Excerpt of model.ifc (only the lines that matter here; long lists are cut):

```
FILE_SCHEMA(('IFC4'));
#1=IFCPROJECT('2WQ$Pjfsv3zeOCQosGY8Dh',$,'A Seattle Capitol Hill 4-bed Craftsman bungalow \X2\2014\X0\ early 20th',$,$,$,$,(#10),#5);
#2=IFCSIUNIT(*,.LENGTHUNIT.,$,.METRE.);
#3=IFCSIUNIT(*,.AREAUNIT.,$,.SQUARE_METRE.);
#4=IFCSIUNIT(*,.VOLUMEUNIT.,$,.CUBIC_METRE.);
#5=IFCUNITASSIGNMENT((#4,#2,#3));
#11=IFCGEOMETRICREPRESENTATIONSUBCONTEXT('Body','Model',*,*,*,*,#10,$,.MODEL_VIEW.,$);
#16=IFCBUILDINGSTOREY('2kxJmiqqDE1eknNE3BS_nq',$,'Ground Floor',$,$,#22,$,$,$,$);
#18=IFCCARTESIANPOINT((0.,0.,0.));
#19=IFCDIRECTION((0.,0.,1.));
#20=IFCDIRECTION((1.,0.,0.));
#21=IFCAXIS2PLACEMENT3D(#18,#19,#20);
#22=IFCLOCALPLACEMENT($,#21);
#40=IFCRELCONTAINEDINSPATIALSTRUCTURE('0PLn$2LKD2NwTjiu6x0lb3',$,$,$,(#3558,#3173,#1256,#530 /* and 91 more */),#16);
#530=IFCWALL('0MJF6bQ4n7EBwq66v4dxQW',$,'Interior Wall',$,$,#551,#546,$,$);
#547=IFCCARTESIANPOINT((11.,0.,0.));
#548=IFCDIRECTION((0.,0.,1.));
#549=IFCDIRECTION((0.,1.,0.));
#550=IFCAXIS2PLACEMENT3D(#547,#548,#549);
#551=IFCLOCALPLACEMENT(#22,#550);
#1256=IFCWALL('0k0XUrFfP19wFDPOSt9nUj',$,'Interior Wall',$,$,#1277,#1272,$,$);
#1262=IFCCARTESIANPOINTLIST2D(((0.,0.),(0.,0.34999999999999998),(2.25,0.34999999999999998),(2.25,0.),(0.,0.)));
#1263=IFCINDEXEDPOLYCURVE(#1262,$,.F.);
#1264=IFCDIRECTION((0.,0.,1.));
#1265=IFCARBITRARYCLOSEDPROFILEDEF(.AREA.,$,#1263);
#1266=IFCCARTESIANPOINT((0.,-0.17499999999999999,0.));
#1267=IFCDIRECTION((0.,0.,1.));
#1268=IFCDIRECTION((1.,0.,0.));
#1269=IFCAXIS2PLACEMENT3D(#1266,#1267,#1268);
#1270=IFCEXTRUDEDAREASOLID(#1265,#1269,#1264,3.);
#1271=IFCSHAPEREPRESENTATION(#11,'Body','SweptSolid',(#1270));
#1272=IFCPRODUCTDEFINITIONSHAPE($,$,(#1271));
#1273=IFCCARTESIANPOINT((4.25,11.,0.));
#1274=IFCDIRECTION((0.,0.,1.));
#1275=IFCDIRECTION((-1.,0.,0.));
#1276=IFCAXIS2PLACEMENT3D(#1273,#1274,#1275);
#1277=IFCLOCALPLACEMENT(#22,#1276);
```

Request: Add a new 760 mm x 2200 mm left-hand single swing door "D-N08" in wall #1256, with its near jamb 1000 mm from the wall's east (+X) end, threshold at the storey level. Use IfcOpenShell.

```python
import numpy as np
import ifcopenshell
import ifcopenshell.api.feature
import ifcopenshell.api.geometry
import ifcopenshell.api.root
import ifcopenshell.api.spatial
import ifcopenshell.geom
import ifcopenshell.util.element
import ifcopenshell.util.placement
import ifcopenshell.util.representation
import ifcopenshell.util.shape
import ifcopenshell.util.unit

model = ifcopenshell.open("model.ifc")
unit_scale = ifcopenshell.util.unit.calculate_unit_scale(model)
settings = ifcopenshell.geom.settings()


def volume(element):
    """Net volume in cubic metres, openings subtracted."""
    shape = ifcopenshell.geom.create_shape(settings, element)
    return ifcopenshell.util.shape.get_volume(shape.geometry)


wall = model.by_guid("0k0XUrFfP19wFDPOSt9nUj")
storey = ifcopenshell.util.element.get_container(wall, ifc_class="IfcBuildingStorey")
context = ifcopenshell.util.representation.get_context(model, "Model", "Body", "MODEL_VIEW")
before = volume(wall)

width, height, from_end, sill = 0.76, 2.2, 1, 0.0  # metres

# The wall runs along its own X axis, and the end named is its -X end.
wall_shape = ifcopenshell.geom.create_shape(settings, wall)
x, y, z = ifcopenshell.util.shape.get_vertices(wall_shape.geometry).T
start = x.min() + from_end
face, thickness = float(y.min()), float(y.max() - y.min())
wall_matrix = ifcopenshell.util.placement.get_local_placement(wall.ObjectPlacement)
level = ifcopenshell.util.placement.get_local_placement(storey.ObjectPlacement)[2, 3]


def in_wall(x, y):
    """Placement at x, y metres in the wall's axes, at sill height."""
    matrix = wall_matrix.copy()
    matrix[:, 3] = wall_matrix @ np.array([x / unit_scale, y / unit_scale, 0.0, 1.0])
    matrix[2, 3] = level + sill / unit_scale
    return matrix


# Opening: a box that overshoots both wall faces by 50 mm.
opening = ifcopenshell.api.root.create_entity(model, ifc_class="IfcOpeningElement", predefined_type="OPENING")
box = ifcopenshell.api.geometry.add_wall_representation(
    model, context=context, length=width, height=height, thickness=thickness + 0.1
)
ifcopenshell.api.geometry.assign_representation(model, product=opening, representation=box)
ifcopenshell.api.geometry.edit_object_placement(model, product=opening, matrix=in_wall(start, face - 0.05), is_si=False)
ifcopenshell.api.feature.add_feature(model, feature=opening, element=wall)

door = ifcopenshell.api.root.create_entity(model, ifc_class="IfcDoor", name="D-N08", predefined_type="DOOR")
door.OverallWidth, door.OverallHeight = width / unit_scale, height / unit_scale
door.OperationType = "SINGLE_SWING_LEFT"
body = ifcopenshell.api.geometry.add_door_representation(
    model,
    context=context,
    overall_width=door.OverallWidth,
    overall_height=door.OverallHeight,
    operation_type="SINGLE_SWING_LEFT",
    lining_properties={"LiningDepth": thickness / unit_scale, "ThresholdDepth": thickness / unit_scale},
)
ifcopenshell.api.geometry.assign_representation(model, product=door, representation=body)
ifcopenshell.api.spatial.assign_container(model, products=[door], relating_structure=storey)
ifcopenshell.api.feature.add_filling(model, opening=opening, element=door)

# The lining spans the wall, so the door starts at the wall face.
ifcopenshell.api.geometry.edit_object_placement(model, product=door, matrix=in_wall(start, face), is_si=False)

after = volume(wall)

print(f"wall volume {before:.3f} -> {after:.3f} m3")

model.write("model_updated.ifc")
```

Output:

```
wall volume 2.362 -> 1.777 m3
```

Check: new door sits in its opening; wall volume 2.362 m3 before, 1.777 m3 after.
